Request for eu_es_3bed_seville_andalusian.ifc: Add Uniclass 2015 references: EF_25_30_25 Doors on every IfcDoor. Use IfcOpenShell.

First a look at what the model holds.

```python
import ifcopenshell

model = ifcopenshell.open("eu_es_3bed_seville_andalusian.ifc")
print(model.schema)
print("classifications:", [c.Name for c in model.by_type("IfcClassification")])
for ifc_class in ("IfcDoor", "IfcRoof", "IfcStair", "IfcWall", "IfcWindow"):
    print(ifc_class, len(model.by_type(ifc_class)))
```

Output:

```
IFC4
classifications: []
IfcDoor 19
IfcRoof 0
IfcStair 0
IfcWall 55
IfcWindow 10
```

```python
import ifcopenshell
import ifcopenshell.api.classification

model = ifcopenshell.open("eu_es_3bed_seville_andalusian.ifc")

system = ifcopenshell.api.classification.add_classification(model, classification="Uniclass 2015")

codes = {
    "IfcDoor": ("EF_25_30_25", "Doors"),
}
for ifc_class, (code, name) in codes.items():
    products = model.by_type(ifc_class)
    ifcopenshell.api.classification.add_reference(
        model, products=products, classification=system, identification=code, name=name
    )
    print(code, len(products))

model.write("eu_es_3bed_seville_andalusian_v2.ifc")
```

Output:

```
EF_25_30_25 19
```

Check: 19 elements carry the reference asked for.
